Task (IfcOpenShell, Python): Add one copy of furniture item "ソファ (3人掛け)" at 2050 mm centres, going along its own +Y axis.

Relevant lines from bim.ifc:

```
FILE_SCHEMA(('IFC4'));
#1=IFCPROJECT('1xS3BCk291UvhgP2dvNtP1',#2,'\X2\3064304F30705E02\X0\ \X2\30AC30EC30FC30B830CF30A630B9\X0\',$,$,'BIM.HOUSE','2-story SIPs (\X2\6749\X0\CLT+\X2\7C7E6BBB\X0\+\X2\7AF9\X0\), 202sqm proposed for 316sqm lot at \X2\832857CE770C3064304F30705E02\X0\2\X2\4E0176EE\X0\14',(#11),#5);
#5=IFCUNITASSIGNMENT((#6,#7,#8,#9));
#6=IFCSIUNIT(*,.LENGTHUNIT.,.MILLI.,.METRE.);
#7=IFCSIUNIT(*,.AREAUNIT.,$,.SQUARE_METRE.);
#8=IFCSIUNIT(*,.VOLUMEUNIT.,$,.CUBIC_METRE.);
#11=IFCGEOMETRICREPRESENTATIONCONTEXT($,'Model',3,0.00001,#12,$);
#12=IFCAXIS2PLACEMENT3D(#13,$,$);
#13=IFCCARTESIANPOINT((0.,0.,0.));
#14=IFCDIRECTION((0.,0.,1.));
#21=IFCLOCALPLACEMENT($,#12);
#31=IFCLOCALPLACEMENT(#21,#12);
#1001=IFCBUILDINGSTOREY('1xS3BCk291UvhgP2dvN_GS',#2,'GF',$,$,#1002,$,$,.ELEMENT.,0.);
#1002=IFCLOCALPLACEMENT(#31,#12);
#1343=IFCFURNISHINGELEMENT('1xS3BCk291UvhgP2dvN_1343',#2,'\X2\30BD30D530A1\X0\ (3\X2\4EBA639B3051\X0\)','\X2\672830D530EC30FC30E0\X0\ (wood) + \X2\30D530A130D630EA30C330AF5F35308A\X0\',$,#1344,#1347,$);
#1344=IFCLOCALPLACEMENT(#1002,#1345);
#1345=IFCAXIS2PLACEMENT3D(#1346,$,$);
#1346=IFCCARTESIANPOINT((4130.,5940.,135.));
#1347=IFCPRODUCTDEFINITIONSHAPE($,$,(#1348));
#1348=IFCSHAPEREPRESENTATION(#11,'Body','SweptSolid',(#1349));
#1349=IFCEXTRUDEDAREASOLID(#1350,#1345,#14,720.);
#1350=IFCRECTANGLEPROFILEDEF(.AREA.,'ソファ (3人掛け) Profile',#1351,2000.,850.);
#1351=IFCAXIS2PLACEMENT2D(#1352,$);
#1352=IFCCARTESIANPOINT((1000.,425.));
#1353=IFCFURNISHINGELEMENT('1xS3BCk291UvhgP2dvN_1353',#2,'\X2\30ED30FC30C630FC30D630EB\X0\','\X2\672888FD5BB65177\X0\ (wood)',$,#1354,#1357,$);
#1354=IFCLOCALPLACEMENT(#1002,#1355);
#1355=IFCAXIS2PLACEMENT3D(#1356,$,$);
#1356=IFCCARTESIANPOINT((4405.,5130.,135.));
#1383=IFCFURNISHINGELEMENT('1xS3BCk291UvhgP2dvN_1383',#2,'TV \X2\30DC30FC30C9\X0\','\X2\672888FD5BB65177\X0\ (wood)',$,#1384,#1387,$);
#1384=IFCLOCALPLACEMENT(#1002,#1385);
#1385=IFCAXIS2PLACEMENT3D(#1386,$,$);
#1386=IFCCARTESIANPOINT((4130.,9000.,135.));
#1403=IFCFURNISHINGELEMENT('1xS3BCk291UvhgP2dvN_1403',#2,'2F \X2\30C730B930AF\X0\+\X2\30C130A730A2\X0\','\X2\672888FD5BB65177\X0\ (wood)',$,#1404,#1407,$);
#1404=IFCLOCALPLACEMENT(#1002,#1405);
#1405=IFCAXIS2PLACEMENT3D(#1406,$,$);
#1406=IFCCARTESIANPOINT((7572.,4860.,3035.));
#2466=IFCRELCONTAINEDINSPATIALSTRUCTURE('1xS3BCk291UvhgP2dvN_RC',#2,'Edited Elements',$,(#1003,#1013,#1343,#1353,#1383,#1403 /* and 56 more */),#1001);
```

```python
import ifcopenshell
import ifcopenshell.api.geometry
import ifcopenshell.api.root
import ifcopenshell.util.element
import ifcopenshell.util.placement
import ifcopenshell.util.unit

model = ifcopenshell.open("bim.ifc")
unit_scale = ifcopenshell.util.unit.calculate_unit_scale(model)


def reuse_history(source, copy):
    """copy_class also copies each property set's owner history, people and application; keep the originals."""
    for rel in copy.IsDefinedBy:
        if rel.is_a("IfcRelDefinesByProperties") and (history := rel.RelatingPropertyDefinition.OwnerHistory):
            rel.RelatingPropertyDefinition.OwnerHistory = source.OwnerHistory
            ifcopenshell.util.element.remove_deep2(model, history)


source = model.by_guid("1xS3BCk291UvhgP2dvN_1343")
base = ifcopenshell.util.placement.get_local_placement(source.ObjectPlacement)
step = base[:3, 1] * 2.05 / unit_scale

for i in range(1, 2):
    copy = ifcopenshell.api.root.copy_class(model, product=source)
    copy.Representation = ifcopenshell.util.element.copy_deep(
        model, source.Representation, exclude=["IfcGeometricRepresentationContext", "IfcRepresentationMap"]
    )
    reuse_history(source, copy)
    matrix = base.copy()
    matrix[:3, 3] += i * step
    print("added at", matrix[:3, 3].round(3) + 0.0)
    ifcopenshell.api.geometry.edit_object_placement(model, product=copy, matrix=matrix, is_si=False)

model.write("bim_v2.ifc")
```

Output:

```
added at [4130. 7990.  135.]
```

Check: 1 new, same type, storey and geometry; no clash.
